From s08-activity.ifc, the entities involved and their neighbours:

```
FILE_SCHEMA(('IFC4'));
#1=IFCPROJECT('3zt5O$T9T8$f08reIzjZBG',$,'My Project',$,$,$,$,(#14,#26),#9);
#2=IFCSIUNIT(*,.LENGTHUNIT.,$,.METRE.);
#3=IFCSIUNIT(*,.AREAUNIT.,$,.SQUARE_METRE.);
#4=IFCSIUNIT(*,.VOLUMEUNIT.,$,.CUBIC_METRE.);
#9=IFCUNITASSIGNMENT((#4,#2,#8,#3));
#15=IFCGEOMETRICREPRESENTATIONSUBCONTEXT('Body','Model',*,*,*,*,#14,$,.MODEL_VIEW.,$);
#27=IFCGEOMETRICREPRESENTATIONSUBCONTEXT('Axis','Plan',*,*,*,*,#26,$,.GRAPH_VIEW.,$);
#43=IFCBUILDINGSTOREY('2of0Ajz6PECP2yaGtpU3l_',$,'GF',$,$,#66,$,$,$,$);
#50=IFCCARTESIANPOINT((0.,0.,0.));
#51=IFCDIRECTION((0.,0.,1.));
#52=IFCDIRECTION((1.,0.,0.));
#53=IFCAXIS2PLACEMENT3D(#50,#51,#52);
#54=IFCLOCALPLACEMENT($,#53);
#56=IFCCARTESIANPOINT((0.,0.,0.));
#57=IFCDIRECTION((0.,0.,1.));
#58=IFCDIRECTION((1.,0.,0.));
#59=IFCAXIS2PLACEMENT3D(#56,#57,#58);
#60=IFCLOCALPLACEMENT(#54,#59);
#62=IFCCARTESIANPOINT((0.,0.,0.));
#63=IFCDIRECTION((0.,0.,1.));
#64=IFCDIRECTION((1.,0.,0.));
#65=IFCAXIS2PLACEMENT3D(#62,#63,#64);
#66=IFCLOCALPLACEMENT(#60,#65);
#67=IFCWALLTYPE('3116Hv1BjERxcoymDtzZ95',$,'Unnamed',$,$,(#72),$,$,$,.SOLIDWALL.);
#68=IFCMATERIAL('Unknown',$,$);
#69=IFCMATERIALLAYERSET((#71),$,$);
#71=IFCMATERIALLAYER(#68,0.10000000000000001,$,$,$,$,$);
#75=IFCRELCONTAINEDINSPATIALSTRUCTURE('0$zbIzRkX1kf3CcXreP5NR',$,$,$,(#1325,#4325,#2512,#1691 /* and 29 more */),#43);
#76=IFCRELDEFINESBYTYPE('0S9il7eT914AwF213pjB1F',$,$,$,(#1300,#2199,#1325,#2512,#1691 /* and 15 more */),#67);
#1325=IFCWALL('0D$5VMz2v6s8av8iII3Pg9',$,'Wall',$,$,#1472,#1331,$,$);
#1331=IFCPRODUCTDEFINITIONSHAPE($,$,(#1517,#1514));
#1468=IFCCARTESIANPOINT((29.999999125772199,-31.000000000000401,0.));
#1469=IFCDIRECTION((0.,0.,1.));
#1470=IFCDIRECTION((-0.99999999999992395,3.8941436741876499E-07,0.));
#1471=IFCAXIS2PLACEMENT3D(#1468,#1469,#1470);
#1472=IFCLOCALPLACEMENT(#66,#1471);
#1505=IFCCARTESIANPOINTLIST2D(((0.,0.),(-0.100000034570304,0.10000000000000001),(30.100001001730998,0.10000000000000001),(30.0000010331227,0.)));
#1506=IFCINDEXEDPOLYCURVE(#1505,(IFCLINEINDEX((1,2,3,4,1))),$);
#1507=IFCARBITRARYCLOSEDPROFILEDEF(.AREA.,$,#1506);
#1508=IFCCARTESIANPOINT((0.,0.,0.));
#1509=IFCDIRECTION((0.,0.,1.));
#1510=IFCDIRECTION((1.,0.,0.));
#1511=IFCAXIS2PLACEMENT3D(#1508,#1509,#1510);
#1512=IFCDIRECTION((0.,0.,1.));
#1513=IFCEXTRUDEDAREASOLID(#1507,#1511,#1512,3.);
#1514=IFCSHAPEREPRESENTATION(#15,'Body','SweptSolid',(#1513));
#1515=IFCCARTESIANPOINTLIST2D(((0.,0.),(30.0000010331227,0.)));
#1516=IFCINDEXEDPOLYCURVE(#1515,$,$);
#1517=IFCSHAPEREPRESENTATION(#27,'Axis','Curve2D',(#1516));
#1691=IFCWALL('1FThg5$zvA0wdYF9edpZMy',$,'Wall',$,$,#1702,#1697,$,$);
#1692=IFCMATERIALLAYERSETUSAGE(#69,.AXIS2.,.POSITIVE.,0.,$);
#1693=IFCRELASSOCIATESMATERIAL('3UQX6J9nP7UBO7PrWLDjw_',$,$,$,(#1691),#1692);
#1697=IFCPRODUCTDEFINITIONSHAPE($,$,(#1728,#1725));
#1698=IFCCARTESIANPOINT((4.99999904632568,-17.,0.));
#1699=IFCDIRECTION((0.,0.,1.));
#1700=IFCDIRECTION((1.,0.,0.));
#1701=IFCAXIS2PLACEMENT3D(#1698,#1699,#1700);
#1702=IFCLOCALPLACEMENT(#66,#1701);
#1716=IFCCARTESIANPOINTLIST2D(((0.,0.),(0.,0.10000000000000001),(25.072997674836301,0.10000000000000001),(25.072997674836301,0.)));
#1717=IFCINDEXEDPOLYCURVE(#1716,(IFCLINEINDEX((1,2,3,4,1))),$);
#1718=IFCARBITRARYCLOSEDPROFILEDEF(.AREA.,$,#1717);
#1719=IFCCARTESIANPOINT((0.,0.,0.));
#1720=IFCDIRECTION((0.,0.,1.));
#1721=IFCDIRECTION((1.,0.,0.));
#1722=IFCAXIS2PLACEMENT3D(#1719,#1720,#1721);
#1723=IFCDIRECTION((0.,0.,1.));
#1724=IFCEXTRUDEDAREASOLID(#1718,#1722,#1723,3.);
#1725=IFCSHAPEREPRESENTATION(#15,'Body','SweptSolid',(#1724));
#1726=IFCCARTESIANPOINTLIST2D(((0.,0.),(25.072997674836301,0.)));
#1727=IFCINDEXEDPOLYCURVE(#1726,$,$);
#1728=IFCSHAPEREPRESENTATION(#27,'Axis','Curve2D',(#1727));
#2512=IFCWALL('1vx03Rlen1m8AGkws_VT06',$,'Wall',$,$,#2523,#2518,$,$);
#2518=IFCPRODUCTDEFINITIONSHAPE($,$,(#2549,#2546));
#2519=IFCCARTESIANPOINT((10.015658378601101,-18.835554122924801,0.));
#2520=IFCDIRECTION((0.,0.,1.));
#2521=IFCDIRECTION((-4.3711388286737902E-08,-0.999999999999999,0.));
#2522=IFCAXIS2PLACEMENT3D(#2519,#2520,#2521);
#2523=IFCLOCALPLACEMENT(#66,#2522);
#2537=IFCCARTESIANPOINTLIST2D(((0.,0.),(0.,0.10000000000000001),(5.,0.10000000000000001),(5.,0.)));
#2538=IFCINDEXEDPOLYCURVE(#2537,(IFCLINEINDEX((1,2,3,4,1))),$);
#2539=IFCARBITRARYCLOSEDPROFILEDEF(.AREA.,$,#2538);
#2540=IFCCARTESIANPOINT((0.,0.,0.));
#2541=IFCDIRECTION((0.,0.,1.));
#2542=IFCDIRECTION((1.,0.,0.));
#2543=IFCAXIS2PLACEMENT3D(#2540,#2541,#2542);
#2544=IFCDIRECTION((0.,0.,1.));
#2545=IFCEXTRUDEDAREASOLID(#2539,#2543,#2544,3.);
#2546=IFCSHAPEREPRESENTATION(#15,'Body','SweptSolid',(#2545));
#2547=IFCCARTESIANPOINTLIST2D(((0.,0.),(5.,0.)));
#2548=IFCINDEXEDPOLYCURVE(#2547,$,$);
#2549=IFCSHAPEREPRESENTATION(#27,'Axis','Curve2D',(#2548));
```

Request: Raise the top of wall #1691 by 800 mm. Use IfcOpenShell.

```python
import ifcopenshell
import ifcopenshell.geom
import ifcopenshell.util.representation
import ifcopenshell.util.shape
import ifcopenshell.util.unit

model = ifcopenshell.open("s08-activity.ifc")
unit_scale = ifcopenshell.util.unit.calculate_unit_scale(model)
settings = ifcopenshell.geom.settings()


def volume(element):
    """Net volume in cubic metres, openings subtracted."""
    shape = ifcopenshell.geom.create_shape(settings, element)
    return ifcopenshell.util.shape.get_volume(shape.geometry)


wall = model.by_guid("1FThg5$zvA0wdYF9edpZMy")
before = volume(wall)

body = ifcopenshell.util.representation.get_representation(wall, "Model", "Body")
solid = body.Items[0]
old_height = solid.Depth
solid.Depth += 0.8 / unit_scale
after = volume(wall)

print(f"height {old_height:g} -> {solid.Depth:g}, volume {before:.3f} -> {after:.3f} m3")

model.write("s08-activity_rev.ifc")
```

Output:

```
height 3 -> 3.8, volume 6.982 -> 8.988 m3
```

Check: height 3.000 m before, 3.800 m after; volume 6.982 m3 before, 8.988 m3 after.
